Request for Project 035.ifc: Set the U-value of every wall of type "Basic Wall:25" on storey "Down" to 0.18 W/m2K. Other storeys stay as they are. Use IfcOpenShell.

First a look at what the model holds.

```python
import ifcopenshell
import ifcopenshell.util.element

model = ifcopenshell.open("Project 035.ifc")
print(model.schema)
storey = next(s for s in model.by_type("IfcBuildingStorey") if s.Name == "Down")
walls = [e for e in ifcopenshell.util.element.get_decomposition(storey) if e.is_a("IfcWall")]
seen = {}
for e in walls:
    element_type = ifcopenshell.util.element.get_type(e)
    key = (element_type.Name if element_type != e and element_type else None, ifcopenshell.util.element.get_pset(e, "Pset_WallCommon", "ThermalTransmittance"))
    seen[key] = seen.get(key, 0) + 1
for (name, value), count in sorted(seen.items(), key=str):
    print(count, "x", name, "|", value)
```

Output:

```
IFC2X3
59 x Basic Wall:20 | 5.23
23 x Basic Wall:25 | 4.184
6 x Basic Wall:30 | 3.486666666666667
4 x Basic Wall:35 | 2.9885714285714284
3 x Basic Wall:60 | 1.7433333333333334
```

```python
import ifcopenshell
import ifcopenshell.api.pset
import ifcopenshell.util.element

model = ifcopenshell.open("Project 035.ifc")

storey = next(s for s in model.by_type("IfcBuildingStorey") if s.Name == "Down")
walls = [e for e in ifcopenshell.util.element.get_decomposition(storey) if e.is_a("IfcWall")]

count = 0
for e in walls:
    element_type = ifcopenshell.util.element.get_type(e)
    if element_type in (None, e) or element_type.Name != "Basic Wall:25":
        continue
    # add_pset returns the element's existing set when there is one.
    pset = ifcopenshell.api.pset.add_pset(model, product=e, name="Pset_WallCommon")
    ifcopenshell.api.pset.edit_pset(model, pset=pset, properties={"ThermalTransmittance": 0.18})
    count += 1

print(count, "walls updated")

model.write("Project 035-out.ifc")
```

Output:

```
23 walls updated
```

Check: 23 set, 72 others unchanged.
